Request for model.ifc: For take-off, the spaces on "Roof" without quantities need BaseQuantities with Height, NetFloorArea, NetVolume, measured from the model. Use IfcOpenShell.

First a look at what the model holds.

```python
import ifcopenshell
import ifcopenshell.util.element
import ifcopenshell.util.unit

model = ifcopenshell.open("model.ifc")
print(model.schema)
for unit_type in ("LENGTHUNIT", "AREAUNIT", "VOLUMEUNIT"):
    print(unit_type, ifcopenshell.util.unit.calculate_unit_scale(model, unit_type))
storey = next(s for s in model.by_type("IfcBuildingStorey") if s.Name == "Roof")
spaces = [e for e in ifcopenshell.util.element.get_decomposition(storey) if e.is_a("IfcSpace")]
for e in sorted(spaces, key=lambda e: e.id()):
    print(e.id(), e.is_a(), e.Name, list(ifcopenshell.util.element.get_psets(e, qtos_only=True)), sep=" | ")
```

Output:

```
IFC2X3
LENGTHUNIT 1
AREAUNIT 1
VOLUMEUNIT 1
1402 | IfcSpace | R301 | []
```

```python
import ifcopenshell
import ifcopenshell.api.pset
import ifcopenshell.geom
import ifcopenshell.util.element
import ifcopenshell.util.shape
import ifcopenshell.util.unit

model = ifcopenshell.open("model.ifc")
unit_scale = ifcopenshell.util.unit.calculate_unit_scale(model)
area_scale = ifcopenshell.util.unit.calculate_unit_scale(model, "AREAUNIT")
volume_scale = ifcopenshell.util.unit.calculate_unit_scale(model, "VOLUMEUNIT")
settings = ifcopenshell.geom.settings()

storey = next(s for s in model.by_type("IfcBuildingStorey") if s.Name == "Roof")
spaces = [e for e in ifcopenshell.util.element.get_decomposition(storey) if e.is_a("IfcSpace")]

for e in sorted(spaces, key=lambda e: e.id()):
    if ifcopenshell.util.element.get_psets(e, qtos_only=True, should_inherit=False):
        continue
    # Geometry comes back in metres, in the element's own axes.
    shape = ifcopenshell.geom.create_shape(settings, e)
    values = {
        "Height": ifcopenshell.util.shape.get_z(shape.geometry) / unit_scale,
        "NetFloorArea": ifcopenshell.util.shape.get_footprint_area(shape.geometry) / area_scale,
        "NetVolume": ifcopenshell.util.shape.get_volume(shape.geometry) / volume_scale,
    }
    qto = ifcopenshell.api.pset.add_qto(model, product=e, name="BaseQuantities")
    ifcopenshell.api.pset.edit_qto(model, qto=qto, properties=values)
    print(e.id(), {k: round(v, 3) for k, v in values.items()})

model.write("model_v2.ifc")
```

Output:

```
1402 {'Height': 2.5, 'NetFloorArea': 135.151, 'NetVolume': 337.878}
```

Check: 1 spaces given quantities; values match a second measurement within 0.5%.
